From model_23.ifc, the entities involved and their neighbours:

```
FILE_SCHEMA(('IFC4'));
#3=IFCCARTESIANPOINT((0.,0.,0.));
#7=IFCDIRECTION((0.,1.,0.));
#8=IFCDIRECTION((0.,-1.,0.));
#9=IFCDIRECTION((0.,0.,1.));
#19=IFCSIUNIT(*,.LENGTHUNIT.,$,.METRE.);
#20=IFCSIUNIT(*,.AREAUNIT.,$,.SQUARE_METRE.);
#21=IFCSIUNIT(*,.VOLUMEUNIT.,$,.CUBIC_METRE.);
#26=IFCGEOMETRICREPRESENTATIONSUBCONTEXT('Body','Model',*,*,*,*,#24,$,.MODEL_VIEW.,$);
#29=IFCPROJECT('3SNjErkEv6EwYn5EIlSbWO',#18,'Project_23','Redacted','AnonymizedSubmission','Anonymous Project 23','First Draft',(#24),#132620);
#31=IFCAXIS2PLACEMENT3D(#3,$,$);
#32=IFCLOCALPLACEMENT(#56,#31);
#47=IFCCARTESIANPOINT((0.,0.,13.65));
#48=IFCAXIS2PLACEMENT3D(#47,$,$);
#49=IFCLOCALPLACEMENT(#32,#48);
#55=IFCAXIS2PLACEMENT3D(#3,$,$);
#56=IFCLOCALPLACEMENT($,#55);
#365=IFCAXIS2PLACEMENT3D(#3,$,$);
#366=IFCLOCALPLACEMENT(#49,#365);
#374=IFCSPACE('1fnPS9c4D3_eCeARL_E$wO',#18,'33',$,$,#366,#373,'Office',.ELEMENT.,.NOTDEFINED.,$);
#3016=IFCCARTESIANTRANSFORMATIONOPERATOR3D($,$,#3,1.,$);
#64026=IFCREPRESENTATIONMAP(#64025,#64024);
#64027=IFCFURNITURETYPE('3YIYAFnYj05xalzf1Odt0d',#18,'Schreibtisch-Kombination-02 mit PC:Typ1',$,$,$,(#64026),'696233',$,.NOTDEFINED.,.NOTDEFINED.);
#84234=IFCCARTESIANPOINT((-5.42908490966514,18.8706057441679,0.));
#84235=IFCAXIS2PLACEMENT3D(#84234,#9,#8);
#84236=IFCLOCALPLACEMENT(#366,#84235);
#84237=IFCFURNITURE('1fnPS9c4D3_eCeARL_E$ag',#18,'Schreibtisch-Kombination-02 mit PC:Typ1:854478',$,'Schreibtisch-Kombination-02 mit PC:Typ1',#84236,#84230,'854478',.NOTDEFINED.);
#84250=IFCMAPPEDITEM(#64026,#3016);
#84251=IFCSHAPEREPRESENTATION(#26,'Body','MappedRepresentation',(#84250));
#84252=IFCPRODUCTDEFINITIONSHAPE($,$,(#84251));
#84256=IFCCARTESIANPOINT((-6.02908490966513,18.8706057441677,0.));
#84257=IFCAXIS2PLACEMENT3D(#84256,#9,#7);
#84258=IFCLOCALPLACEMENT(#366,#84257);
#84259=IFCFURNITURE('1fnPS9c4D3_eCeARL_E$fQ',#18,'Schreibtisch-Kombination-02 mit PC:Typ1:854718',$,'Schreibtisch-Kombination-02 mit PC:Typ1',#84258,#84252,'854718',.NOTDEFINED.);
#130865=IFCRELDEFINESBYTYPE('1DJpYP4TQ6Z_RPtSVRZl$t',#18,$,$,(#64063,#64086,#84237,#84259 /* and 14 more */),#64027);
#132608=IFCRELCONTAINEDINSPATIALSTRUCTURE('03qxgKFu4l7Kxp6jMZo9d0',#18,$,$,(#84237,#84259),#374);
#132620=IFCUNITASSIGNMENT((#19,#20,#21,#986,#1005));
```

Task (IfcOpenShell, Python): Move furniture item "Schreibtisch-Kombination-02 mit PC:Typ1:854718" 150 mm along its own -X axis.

```python
import ifcopenshell
import ifcopenshell.api.geometry
import ifcopenshell.util.placement
import ifcopenshell.util.unit

model = ifcopenshell.open("model_23.ifc")
unit_scale = ifcopenshell.util.unit.calculate_unit_scale(model)

item = model.by_guid("1fnPS9c4D3_eCeARL_E$fQ")
matrix = ifcopenshell.util.placement.get_local_placement(item.ObjectPlacement)
matrix[:3, 3] -= matrix[:3, 0] * 0.15 / unit_scale
ifcopenshell.api.geometry.edit_object_placement(model, product=item, matrix=matrix, is_si=False)

print(ifcopenshell.util.placement.get_local_placement(item.ObjectPlacement).round(3) + 0.0)

model.write("model_23_v2.ifc")
```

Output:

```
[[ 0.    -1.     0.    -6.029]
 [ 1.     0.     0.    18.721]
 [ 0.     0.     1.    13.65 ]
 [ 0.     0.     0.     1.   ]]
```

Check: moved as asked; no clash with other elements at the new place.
